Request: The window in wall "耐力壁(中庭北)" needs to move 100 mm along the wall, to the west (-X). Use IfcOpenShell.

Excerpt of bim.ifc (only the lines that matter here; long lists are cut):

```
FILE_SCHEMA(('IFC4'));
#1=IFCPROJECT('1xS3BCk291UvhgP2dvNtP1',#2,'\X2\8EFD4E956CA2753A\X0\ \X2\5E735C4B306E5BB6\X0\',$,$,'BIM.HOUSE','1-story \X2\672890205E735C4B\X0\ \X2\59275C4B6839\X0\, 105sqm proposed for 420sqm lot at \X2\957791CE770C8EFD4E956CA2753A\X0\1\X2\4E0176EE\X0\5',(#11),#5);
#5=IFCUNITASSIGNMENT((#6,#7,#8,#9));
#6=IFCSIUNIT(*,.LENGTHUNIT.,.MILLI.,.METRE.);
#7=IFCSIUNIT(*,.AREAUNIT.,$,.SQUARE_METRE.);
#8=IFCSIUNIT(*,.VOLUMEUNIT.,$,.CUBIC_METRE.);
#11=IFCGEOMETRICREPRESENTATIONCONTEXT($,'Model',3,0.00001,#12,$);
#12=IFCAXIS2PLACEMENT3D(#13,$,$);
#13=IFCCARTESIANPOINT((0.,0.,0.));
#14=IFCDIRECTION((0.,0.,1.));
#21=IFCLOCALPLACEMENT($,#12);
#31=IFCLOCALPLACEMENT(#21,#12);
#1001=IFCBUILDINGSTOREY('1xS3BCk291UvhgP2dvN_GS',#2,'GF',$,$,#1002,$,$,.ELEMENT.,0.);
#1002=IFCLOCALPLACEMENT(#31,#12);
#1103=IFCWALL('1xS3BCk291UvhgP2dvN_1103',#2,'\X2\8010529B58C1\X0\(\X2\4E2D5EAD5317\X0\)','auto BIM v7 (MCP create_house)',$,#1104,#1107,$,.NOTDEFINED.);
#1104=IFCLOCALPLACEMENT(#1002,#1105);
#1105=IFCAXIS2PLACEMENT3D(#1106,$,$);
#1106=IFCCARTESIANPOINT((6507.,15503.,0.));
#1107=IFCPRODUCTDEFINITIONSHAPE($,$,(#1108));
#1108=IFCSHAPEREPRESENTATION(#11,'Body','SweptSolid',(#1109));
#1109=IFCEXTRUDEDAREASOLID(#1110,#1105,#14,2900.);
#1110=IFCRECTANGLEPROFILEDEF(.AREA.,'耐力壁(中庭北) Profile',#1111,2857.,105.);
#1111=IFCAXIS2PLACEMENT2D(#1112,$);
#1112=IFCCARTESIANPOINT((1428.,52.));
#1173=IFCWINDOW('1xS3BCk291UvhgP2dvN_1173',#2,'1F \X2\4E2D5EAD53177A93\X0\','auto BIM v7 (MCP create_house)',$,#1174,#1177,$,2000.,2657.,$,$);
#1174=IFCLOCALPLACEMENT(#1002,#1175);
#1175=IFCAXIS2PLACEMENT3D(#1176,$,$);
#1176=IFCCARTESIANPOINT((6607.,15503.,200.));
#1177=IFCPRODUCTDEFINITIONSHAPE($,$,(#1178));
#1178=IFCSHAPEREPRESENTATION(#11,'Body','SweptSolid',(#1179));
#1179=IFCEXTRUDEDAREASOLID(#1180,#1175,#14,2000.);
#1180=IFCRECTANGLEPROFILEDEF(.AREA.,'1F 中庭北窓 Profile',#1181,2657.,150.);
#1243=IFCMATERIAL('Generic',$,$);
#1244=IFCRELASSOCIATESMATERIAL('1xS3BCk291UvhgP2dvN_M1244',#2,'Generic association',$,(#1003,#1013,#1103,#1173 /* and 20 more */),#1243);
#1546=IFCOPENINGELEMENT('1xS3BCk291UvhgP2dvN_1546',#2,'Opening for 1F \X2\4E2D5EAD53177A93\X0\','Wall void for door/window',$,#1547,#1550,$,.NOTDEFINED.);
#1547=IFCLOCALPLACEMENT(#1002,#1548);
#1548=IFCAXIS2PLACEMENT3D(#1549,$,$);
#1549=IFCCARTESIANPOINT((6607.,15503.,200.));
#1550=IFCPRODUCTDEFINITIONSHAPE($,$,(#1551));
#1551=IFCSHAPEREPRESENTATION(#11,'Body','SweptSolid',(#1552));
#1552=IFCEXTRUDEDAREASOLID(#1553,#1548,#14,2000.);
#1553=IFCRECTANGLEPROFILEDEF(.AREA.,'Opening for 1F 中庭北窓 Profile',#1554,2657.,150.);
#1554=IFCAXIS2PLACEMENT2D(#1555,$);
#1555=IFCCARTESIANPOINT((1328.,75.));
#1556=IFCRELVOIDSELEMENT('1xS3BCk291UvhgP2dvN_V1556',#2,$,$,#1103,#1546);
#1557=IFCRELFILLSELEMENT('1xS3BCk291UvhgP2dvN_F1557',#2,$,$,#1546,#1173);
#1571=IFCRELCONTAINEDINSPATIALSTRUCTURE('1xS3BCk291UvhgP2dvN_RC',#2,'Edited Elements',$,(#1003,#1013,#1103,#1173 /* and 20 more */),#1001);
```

```python
import ifcopenshell
import ifcopenshell.api.geometry
import ifcopenshell.util.placement
import ifcopenshell.util.unit

model = ifcopenshell.open("bim.ifc")
unit_scale = ifcopenshell.util.unit.calculate_unit_scale(model)

window = model.by_guid("1xS3BCk291UvhgP2dvN_1173")
opening = window.FillsVoids[0].RelatingOpeningElement
wall = opening.VoidsElements[0].RelatingBuildingElement

wall_matrix = ifcopenshell.util.placement.get_local_placement(wall.ObjectPlacement)
shift = wall_matrix[:3, 0] * -0.1 / unit_scale
before = ifcopenshell.util.placement.get_local_placement(window.ObjectPlacement)[:3, 3].copy()

# The window is not placed relative to its opening, so move both.
for product in (opening, window):
    matrix = ifcopenshell.util.placement.get_local_placement(product.ObjectPlacement)
    matrix[:3, 3] += shift
    ifcopenshell.api.geometry.edit_object_placement(model, product=product, matrix=matrix, is_si=False)

after = ifcopenshell.util.placement.get_local_placement(window.ObjectPlacement)[:3, 3]
print("window moved by", (after - before).round(3) + 0.0)

model.write("bim_v2.ifc")
```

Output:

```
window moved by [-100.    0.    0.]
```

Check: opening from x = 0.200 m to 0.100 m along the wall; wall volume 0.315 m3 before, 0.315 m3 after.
